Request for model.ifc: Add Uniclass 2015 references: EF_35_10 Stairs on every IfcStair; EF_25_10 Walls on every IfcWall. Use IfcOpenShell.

First a look at what the model holds.

```python
import ifcopenshell

model = ifcopenshell.open("model.ifc")
print(model.schema)
print("classifications:", [c.Name for c in model.by_type("IfcClassification")])
for ifc_class in ("IfcDoor", "IfcRoof", "IfcStair", "IfcWall", "IfcWindow"):
    print(ifc_class, len(model.by_type(ifc_class)))
```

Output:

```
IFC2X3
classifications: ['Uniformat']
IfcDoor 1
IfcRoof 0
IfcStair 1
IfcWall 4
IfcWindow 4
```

```python
import ifcopenshell
import ifcopenshell.api.classification

model = ifcopenshell.open("model.ifc")

# IFC2X3 requires Source and Edition and has no link from the project to the system.
system = model.create_entity("IfcClassification", Source="NBS", Edition="2015", Name="Uniclass 2015")

codes = {
    "IfcStair": ("EF_35_10", "Stairs"),
    "IfcWall": ("EF_25_10", "Walls"),
}
for ifc_class, (code, name) in codes.items():
    products = model.by_type(ifc_class)
    ifcopenshell.api.classification.add_reference(
        model, products=products, classification=system, identification=code, name=name
    )
    print(code, len(products))

model.write("model_rev.ifc")
```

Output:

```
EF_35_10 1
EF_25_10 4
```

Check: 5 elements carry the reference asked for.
